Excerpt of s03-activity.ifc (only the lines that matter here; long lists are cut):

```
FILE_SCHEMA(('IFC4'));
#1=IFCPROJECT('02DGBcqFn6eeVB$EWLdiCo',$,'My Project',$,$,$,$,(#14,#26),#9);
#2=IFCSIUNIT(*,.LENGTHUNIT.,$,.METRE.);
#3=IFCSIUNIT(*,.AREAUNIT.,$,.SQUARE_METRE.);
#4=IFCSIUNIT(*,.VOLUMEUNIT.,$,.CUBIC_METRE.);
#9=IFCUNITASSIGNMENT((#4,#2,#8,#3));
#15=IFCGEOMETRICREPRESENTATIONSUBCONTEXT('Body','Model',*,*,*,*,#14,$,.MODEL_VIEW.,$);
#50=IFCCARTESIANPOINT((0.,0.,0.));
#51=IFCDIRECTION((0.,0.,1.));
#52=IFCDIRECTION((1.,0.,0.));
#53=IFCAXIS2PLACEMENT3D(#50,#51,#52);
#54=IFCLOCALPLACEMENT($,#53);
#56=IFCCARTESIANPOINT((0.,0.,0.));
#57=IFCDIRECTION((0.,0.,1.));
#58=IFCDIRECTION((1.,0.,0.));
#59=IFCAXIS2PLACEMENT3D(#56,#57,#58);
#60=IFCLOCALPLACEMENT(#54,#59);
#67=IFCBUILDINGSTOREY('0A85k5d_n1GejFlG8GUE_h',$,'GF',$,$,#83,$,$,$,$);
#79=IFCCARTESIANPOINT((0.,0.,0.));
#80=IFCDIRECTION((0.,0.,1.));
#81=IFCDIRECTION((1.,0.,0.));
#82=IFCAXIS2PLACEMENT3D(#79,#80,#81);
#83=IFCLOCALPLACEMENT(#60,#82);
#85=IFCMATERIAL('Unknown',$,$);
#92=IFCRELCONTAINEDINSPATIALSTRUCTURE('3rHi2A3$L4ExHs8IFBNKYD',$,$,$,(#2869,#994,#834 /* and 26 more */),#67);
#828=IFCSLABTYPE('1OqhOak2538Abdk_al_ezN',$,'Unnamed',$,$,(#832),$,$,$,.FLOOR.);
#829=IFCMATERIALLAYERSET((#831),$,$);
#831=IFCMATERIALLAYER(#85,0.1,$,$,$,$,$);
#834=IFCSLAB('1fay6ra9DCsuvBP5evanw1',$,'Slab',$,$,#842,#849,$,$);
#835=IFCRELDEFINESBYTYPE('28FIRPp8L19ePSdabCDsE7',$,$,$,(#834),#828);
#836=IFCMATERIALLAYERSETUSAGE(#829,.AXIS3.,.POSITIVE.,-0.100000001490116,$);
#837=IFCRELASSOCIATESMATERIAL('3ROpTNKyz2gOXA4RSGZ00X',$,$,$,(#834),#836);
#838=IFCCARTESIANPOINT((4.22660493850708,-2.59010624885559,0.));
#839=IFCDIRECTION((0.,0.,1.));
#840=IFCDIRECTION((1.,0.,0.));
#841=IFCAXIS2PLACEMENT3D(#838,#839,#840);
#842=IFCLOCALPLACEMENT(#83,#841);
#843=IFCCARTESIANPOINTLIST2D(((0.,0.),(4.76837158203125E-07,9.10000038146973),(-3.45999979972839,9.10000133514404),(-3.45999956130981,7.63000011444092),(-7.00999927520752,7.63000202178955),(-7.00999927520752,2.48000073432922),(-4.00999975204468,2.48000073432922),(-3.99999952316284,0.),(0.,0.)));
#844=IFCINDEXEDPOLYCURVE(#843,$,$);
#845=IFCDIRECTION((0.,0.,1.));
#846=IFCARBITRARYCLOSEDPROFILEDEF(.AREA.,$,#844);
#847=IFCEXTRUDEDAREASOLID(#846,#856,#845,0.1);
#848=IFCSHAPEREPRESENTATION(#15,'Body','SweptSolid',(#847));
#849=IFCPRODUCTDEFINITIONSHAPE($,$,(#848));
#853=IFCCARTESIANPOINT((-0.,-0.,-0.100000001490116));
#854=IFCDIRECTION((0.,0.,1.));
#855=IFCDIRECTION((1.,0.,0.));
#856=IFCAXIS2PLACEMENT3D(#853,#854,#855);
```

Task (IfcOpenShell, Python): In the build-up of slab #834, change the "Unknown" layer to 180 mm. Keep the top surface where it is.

```python
import ifcopenshell
import ifcopenshell.util.element
import ifcopenshell.util.representation
import ifcopenshell.util.unit

model = ifcopenshell.open("s03-activity.ifc")
unit_scale = ifcopenshell.util.unit.calculate_unit_scale(model)

layer_set = model.by_id(829)
layer = next(l for l in layer_set.MaterialLayers if l.Material and l.Material.Name == "Unknown")
change = 0.18 / unit_scale - layer.LayerThickness
layer.LayerThickness += change

# Geometry does not follow the layer set by itself.
slabs = [e for e in ifcopenshell.util.element.get_elements_by_material(model, layer_set) if e.is_a("IfcSlab")]
for slab in sorted(slabs, key=lambda e: e.id()):
    body = ifcopenshell.util.representation.get_representation(slab, "Model", "Body")
    solid = body.Items[0]
    old_depth = solid.Depth
    solid.Depth += change
    # Extruded upwards: lower the start of the extrusion so the top stays.
    x, y, z = solid.Position.Location.Coordinates
    solid.Position.Location = model.createIfcCartesianPoint((x, y, z - change))
    print(slab.id(), f"{old_depth:g} -> {solid.Depth:g}")

# The layers are counted up from the underside, which has moved.
for usage in {ifcopenshell.util.element.get_material(slab) for slab in slabs}:
    usage.OffsetFromReferenceLine -= change

model.write("s03-activity_edited.ifc")
```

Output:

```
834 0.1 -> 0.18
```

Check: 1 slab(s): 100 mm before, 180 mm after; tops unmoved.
